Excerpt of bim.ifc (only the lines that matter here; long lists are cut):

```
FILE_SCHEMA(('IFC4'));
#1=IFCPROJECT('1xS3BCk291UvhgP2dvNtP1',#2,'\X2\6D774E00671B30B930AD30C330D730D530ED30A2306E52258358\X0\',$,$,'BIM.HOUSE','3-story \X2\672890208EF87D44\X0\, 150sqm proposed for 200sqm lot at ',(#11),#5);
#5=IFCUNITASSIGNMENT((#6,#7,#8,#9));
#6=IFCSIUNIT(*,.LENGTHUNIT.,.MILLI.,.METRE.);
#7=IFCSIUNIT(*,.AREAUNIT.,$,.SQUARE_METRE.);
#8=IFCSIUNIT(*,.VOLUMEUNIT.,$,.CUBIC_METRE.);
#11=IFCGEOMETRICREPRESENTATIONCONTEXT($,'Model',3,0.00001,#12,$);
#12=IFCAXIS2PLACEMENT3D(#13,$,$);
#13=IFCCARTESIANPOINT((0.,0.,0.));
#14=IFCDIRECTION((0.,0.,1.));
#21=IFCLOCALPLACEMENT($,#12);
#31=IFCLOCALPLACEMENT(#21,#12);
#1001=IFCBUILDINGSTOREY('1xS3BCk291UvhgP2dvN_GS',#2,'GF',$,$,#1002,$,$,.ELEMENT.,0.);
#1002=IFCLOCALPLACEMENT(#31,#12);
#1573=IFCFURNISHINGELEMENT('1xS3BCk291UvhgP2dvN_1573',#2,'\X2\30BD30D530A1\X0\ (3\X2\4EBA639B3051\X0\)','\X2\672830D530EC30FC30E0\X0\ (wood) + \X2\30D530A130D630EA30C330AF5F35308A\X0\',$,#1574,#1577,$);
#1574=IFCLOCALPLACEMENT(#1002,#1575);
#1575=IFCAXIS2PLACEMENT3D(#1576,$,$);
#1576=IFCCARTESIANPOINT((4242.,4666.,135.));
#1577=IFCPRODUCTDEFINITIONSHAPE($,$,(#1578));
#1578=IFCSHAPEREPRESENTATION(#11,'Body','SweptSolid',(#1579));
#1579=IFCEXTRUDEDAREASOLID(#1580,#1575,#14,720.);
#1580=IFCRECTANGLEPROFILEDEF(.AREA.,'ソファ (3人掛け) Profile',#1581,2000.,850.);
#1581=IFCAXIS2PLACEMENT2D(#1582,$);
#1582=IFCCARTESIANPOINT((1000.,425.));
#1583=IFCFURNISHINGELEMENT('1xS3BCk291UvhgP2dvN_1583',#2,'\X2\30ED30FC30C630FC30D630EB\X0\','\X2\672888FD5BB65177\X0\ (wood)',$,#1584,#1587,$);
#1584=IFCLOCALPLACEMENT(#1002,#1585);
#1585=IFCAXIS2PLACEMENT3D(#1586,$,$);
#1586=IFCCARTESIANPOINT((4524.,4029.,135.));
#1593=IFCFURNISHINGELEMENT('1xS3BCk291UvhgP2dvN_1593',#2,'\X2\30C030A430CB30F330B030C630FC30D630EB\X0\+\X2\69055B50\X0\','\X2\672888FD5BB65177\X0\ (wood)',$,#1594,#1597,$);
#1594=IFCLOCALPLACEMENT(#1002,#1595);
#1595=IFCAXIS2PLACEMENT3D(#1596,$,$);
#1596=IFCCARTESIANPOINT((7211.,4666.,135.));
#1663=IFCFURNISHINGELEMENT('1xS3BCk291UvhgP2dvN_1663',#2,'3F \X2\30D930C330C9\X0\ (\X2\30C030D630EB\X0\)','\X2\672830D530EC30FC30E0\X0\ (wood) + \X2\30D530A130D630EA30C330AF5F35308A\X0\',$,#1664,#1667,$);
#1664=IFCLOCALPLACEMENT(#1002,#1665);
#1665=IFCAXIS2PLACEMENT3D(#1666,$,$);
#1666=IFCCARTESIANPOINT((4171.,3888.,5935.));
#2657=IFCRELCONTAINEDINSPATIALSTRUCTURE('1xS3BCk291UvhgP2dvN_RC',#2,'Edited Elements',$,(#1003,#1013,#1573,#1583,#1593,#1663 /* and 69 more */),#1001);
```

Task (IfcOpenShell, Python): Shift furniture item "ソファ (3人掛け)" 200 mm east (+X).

```python
import ifcopenshell
import ifcopenshell.api.geometry
import ifcopenshell.util.placement
import ifcopenshell.util.unit

model = ifcopenshell.open("bim.ifc")
unit_scale = ifcopenshell.util.unit.calculate_unit_scale(model)

item = model.by_id(1573)
matrix = ifcopenshell.util.placement.get_local_placement(item.ObjectPlacement)
matrix[0, 3] += 0.2 / unit_scale
ifcopenshell.api.geometry.edit_object_placement(model, product=item, matrix=matrix, is_si=False)

print(ifcopenshell.util.placement.get_local_placement(item.ObjectPlacement).round(3) + 0.0)

model.write("bim_v2.ifc")
```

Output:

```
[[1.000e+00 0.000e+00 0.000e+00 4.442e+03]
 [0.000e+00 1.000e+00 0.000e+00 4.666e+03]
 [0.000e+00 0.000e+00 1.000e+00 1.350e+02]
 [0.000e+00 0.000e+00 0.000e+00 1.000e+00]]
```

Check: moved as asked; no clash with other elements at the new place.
